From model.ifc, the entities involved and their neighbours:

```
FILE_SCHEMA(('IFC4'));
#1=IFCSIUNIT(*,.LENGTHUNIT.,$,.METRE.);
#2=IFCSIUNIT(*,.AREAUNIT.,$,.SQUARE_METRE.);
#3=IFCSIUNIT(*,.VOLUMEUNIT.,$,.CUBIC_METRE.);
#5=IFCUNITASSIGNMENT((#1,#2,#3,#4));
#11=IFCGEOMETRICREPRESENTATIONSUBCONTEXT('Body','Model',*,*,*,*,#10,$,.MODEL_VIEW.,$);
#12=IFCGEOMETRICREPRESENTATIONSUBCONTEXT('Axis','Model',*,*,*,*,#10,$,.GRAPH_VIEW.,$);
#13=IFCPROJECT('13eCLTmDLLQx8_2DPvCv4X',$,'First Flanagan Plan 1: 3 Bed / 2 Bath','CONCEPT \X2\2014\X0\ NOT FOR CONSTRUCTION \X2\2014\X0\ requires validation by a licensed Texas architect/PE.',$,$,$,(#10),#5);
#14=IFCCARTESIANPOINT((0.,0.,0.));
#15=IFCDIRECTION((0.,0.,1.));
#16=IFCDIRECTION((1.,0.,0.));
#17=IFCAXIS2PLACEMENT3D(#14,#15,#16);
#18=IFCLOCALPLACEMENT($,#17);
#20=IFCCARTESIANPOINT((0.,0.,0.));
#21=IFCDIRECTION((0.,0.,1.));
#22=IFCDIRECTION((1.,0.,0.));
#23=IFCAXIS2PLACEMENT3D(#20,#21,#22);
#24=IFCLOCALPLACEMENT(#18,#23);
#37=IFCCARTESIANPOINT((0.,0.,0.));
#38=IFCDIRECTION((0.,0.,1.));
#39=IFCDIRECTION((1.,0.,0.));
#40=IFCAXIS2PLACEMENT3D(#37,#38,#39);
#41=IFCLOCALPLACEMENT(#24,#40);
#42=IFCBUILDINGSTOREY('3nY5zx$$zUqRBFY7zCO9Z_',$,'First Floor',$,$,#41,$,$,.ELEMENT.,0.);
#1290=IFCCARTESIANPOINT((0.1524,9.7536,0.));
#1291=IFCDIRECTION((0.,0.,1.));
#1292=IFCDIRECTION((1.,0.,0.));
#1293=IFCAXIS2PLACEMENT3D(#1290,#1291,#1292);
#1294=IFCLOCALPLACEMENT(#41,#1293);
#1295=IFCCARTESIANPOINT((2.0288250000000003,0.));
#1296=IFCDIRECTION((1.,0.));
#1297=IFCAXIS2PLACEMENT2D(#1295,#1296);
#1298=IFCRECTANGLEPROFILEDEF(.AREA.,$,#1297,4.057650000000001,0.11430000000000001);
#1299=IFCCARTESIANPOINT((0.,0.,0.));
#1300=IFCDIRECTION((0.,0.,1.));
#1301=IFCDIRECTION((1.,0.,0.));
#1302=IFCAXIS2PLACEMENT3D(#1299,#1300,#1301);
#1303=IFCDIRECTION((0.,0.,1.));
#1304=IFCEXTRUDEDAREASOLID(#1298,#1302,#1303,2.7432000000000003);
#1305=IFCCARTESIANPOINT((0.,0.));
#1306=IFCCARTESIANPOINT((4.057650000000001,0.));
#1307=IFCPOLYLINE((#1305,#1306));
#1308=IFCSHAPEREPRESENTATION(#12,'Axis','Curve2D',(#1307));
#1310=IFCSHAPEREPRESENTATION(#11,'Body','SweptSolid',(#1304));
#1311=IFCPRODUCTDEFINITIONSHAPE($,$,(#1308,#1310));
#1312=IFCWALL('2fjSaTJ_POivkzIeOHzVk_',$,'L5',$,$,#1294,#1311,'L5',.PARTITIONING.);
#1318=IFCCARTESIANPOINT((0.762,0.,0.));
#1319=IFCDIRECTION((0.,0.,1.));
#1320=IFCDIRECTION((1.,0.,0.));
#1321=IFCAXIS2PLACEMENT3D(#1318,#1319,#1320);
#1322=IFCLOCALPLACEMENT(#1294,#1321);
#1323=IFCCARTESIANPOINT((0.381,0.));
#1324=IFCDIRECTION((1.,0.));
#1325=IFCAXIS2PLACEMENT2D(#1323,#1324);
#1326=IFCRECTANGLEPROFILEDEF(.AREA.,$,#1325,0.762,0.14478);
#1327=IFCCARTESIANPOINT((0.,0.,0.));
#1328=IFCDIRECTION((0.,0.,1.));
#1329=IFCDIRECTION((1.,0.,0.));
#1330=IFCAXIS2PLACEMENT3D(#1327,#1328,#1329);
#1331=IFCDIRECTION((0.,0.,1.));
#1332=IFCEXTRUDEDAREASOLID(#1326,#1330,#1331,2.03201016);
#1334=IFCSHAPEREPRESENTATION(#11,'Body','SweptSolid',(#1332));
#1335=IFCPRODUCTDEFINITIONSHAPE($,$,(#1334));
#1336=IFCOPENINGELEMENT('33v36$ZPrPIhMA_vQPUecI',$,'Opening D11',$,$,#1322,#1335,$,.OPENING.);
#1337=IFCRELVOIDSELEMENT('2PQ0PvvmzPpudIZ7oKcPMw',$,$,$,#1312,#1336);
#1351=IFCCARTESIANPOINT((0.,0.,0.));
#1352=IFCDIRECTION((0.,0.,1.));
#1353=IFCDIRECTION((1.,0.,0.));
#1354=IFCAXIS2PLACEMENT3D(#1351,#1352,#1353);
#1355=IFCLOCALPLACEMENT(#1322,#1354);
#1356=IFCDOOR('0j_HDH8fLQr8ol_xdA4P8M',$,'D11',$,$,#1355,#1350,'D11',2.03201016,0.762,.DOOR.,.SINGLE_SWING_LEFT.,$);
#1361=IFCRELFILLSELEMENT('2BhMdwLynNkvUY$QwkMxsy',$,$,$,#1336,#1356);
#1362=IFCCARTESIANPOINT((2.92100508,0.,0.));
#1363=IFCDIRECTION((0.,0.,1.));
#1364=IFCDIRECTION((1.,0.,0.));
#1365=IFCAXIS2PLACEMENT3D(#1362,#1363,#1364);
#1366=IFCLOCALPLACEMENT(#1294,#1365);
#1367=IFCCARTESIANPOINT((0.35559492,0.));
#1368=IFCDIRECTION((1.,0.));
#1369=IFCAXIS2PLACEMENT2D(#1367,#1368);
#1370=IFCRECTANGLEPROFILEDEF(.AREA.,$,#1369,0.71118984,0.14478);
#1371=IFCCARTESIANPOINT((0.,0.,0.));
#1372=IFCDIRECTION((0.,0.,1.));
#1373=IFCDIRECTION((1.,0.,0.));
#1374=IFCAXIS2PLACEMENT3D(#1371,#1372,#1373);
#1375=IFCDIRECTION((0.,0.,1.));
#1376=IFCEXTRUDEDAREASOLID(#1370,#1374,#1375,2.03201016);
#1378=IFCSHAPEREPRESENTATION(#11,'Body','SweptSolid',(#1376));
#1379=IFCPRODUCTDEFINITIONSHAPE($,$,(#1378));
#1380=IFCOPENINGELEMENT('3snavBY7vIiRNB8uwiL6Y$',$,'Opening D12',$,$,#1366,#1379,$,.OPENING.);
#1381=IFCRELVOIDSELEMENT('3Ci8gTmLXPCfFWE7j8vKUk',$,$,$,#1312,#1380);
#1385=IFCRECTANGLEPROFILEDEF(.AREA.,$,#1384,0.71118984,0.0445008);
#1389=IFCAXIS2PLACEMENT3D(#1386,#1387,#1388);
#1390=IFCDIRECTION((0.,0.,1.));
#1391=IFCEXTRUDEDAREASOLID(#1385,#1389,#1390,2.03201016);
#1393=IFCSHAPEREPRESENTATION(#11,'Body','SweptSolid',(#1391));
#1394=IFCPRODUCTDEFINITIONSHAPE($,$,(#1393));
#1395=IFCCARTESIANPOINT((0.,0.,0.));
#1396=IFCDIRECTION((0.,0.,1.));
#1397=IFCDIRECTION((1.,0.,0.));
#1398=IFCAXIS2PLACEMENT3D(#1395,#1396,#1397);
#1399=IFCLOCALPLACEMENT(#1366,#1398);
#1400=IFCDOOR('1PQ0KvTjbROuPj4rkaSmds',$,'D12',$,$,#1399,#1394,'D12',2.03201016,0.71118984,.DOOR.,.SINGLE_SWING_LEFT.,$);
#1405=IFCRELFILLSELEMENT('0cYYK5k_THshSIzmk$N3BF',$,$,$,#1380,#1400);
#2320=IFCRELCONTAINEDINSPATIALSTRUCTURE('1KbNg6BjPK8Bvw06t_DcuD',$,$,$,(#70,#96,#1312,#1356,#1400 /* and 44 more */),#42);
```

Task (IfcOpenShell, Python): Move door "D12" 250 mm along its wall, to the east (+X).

```python
import ifcopenshell
import ifcopenshell.api.geometry
import ifcopenshell.util.placement
import ifcopenshell.util.unit

model = ifcopenshell.open("model.ifc")
unit_scale = ifcopenshell.util.unit.calculate_unit_scale(model)

door = model.by_id(1400)
opening = door.FillsVoids[0].RelatingOpeningElement
wall = opening.VoidsElements[0].RelatingBuildingElement

wall_matrix = ifcopenshell.util.placement.get_local_placement(wall.ObjectPlacement)
shift = wall_matrix[:3, 0] * 0.25 / unit_scale
before = ifcopenshell.util.placement.get_local_placement(door.ObjectPlacement)[:3, 3].copy()

# The door is placed relative to its opening, so it follows when the opening moves.
matrix = ifcopenshell.util.placement.get_local_placement(opening.ObjectPlacement)
matrix[:3, 3] += shift
ifcopenshell.api.geometry.edit_object_placement(
    model, product=opening, matrix=matrix, is_si=False, should_transform_children=True
)

after = ifcopenshell.util.placement.get_local_placement(door.ObjectPlacement)[:3, 3]
print("door moved by", (after - before).round(3) + 0.0)

model.write("model_edited.ifc")
```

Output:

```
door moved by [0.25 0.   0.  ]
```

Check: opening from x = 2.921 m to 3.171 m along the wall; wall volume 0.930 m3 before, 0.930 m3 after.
